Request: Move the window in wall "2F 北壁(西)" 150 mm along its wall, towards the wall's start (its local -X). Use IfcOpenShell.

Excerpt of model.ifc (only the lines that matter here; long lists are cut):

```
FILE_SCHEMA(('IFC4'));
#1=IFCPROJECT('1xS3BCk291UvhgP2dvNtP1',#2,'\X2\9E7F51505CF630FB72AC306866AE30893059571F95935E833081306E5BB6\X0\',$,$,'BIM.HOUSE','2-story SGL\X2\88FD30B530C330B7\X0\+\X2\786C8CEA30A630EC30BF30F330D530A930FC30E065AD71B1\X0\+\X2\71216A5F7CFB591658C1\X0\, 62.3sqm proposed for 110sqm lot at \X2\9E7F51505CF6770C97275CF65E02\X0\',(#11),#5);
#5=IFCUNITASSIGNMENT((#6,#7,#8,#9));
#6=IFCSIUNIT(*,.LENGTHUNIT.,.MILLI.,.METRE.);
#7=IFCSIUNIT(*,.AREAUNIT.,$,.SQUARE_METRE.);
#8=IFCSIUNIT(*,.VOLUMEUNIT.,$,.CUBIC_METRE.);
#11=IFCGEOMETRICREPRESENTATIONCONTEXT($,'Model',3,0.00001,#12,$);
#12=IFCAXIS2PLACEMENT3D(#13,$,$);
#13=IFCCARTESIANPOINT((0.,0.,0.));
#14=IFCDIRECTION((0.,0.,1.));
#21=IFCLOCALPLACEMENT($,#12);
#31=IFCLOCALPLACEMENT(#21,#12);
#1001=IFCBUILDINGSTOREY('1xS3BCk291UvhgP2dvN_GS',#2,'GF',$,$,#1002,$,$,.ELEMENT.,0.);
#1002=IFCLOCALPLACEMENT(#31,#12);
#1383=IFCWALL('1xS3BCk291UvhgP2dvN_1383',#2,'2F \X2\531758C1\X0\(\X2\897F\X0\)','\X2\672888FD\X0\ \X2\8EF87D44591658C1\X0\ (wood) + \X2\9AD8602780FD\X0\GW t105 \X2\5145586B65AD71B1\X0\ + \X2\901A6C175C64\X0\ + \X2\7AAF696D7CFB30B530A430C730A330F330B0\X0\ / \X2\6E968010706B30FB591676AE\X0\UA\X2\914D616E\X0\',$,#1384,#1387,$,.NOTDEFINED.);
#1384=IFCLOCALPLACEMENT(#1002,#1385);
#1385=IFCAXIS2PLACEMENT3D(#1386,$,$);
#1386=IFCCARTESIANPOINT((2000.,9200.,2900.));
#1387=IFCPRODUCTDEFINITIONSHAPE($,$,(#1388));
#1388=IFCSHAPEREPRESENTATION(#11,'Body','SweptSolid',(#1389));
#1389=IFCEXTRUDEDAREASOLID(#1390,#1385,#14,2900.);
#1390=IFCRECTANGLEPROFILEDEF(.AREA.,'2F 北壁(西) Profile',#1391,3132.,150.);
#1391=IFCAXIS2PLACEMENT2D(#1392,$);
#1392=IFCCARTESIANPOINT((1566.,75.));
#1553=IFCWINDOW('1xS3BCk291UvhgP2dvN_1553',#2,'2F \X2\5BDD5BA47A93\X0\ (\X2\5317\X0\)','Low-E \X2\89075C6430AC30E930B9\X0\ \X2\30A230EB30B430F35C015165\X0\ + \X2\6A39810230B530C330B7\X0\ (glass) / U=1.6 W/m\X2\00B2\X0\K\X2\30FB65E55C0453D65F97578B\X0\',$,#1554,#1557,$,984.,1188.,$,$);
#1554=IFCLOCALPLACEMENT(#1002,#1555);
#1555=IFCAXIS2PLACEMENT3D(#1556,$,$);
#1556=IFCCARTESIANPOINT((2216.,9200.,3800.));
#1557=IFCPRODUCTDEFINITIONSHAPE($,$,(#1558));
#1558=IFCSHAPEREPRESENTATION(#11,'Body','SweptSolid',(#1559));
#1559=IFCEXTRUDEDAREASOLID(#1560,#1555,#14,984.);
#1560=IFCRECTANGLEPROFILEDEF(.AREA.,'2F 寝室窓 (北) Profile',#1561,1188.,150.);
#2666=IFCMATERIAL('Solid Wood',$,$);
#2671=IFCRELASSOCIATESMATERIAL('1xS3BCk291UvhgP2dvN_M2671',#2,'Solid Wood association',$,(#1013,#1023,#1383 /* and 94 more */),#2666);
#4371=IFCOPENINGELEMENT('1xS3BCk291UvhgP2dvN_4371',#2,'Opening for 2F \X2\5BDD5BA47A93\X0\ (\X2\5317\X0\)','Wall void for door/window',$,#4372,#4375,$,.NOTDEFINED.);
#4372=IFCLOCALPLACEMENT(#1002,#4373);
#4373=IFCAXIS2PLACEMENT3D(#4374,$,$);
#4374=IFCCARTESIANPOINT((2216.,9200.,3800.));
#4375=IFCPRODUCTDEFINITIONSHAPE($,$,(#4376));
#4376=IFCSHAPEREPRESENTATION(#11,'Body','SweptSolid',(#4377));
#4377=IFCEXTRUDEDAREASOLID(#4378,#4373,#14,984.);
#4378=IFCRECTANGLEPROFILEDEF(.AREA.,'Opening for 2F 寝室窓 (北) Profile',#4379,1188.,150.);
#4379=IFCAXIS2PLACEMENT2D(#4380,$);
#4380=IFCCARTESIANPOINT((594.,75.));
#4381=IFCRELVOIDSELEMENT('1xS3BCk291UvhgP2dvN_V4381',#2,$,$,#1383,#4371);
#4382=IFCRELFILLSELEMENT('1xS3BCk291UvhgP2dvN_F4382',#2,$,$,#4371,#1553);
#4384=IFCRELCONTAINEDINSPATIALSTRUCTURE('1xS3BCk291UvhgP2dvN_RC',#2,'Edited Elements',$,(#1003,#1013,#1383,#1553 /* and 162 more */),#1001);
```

```python
import ifcopenshell
import ifcopenshell.api.geometry
import ifcopenshell.util.placement
import ifcopenshell.util.unit

model = ifcopenshell.open("model.ifc")
unit_scale = ifcopenshell.util.unit.calculate_unit_scale(model)

window = model.by_guid("1xS3BCk291UvhgP2dvN_1553")
opening = window.FillsVoids[0].RelatingOpeningElement
wall = opening.VoidsElements[0].RelatingBuildingElement

wall_matrix = ifcopenshell.util.placement.get_local_placement(wall.ObjectPlacement)
shift = wall_matrix[:3, 0] * -0.15 / unit_scale
before = ifcopenshell.util.placement.get_local_placement(window.ObjectPlacement)[:3, 3].copy()

# The window is not placed relative to its opening, so move both.
for product in (opening, window):
    matrix = ifcopenshell.util.placement.get_local_placement(product.ObjectPlacement)
    matrix[:3, 3] += shift
    ifcopenshell.api.geometry.edit_object_placement(model, product=product, matrix=matrix, is_si=False)

after = ifcopenshell.util.placement.get_local_placement(window.ObjectPlacement)[:3, 3]
print("window moved by", (after - before).round(3) + 0.0)

model.write("model_rev.ifc")
```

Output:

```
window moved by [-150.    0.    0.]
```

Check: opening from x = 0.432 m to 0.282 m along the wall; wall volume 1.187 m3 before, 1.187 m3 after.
